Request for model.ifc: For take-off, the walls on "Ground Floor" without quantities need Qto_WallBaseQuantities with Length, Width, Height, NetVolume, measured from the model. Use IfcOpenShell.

First a look at what the model holds.

```python
import ifcopenshell
import ifcopenshell.util.element
import ifcopenshell.util.unit

model = ifcopenshell.open("model.ifc")
print(model.schema)
for unit_type in ("LENGTHUNIT", "AREAUNIT", "VOLUMEUNIT"):
    print(unit_type, ifcopenshell.util.unit.calculate_unit_scale(model, unit_type))
storey = next(s for s in model.by_type("IfcBuildingStorey") if s.Name == "Ground Floor")
walls = [e for e in ifcopenshell.util.element.get_decomposition(storey) if e.is_a("IfcWall")]
for e in sorted(walls, key=lambda e: e.id()):
    print(e.id(), e.is_a(), e.Name, list(ifcopenshell.util.element.get_psets(e, qtos_only=True)), sep=" | ")
```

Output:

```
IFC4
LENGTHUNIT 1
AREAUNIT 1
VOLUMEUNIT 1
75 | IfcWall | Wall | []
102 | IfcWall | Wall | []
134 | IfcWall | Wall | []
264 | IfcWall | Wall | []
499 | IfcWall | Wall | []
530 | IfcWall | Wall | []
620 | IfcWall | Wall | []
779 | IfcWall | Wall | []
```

```python
import ifcopenshell
import ifcopenshell.api.pset
import ifcopenshell.geom
import ifcopenshell.util.element
import ifcopenshell.util.shape
import ifcopenshell.util.unit

model = ifcopenshell.open("model.ifc")
unit_scale = ifcopenshell.util.unit.calculate_unit_scale(model)
volume_scale = ifcopenshell.util.unit.calculate_unit_scale(model, "VOLUMEUNIT")
settings = ifcopenshell.geom.settings()

storey = next(s for s in model.by_type("IfcBuildingStorey") if s.Name == "Ground Floor")
walls = [e for e in ifcopenshell.util.element.get_decomposition(storey) if e.is_a("IfcWall")]

for e in sorted(walls, key=lambda e: e.id()):
    if ifcopenshell.util.element.get_psets(e, qtos_only=True, should_inherit=False):
        continue
    # Geometry comes back in metres, in the element's own axes.
    shape = ifcopenshell.geom.create_shape(settings, e)
    values = {
        "Length": ifcopenshell.util.shape.get_x(shape.geometry) / unit_scale,
        "Width": ifcopenshell.util.shape.get_y(shape.geometry) / unit_scale,
        "Height": ifcopenshell.util.shape.get_z(shape.geometry) / unit_scale,
        "NetVolume": ifcopenshell.util.shape.get_volume(shape.geometry) / volume_scale,
    }
    qto = ifcopenshell.api.pset.add_qto(model, product=e, name="Qto_WallBaseQuantities")
    ifcopenshell.api.pset.edit_qto(model, qto=qto, properties=values)
    print(e.id(), {k: round(v, 3) for k, v in values.items()})

model.write("model_rev.ifc")
```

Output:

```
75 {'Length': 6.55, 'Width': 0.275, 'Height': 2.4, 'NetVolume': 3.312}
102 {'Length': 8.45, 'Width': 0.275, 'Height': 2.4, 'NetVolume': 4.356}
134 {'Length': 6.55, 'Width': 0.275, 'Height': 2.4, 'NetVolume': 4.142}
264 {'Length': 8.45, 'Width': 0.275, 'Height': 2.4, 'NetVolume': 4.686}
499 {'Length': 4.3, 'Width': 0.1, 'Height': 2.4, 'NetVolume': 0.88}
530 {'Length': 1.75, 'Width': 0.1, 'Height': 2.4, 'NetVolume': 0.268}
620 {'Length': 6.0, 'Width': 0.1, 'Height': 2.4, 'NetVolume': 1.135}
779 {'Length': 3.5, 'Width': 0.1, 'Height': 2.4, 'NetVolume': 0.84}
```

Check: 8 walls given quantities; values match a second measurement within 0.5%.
